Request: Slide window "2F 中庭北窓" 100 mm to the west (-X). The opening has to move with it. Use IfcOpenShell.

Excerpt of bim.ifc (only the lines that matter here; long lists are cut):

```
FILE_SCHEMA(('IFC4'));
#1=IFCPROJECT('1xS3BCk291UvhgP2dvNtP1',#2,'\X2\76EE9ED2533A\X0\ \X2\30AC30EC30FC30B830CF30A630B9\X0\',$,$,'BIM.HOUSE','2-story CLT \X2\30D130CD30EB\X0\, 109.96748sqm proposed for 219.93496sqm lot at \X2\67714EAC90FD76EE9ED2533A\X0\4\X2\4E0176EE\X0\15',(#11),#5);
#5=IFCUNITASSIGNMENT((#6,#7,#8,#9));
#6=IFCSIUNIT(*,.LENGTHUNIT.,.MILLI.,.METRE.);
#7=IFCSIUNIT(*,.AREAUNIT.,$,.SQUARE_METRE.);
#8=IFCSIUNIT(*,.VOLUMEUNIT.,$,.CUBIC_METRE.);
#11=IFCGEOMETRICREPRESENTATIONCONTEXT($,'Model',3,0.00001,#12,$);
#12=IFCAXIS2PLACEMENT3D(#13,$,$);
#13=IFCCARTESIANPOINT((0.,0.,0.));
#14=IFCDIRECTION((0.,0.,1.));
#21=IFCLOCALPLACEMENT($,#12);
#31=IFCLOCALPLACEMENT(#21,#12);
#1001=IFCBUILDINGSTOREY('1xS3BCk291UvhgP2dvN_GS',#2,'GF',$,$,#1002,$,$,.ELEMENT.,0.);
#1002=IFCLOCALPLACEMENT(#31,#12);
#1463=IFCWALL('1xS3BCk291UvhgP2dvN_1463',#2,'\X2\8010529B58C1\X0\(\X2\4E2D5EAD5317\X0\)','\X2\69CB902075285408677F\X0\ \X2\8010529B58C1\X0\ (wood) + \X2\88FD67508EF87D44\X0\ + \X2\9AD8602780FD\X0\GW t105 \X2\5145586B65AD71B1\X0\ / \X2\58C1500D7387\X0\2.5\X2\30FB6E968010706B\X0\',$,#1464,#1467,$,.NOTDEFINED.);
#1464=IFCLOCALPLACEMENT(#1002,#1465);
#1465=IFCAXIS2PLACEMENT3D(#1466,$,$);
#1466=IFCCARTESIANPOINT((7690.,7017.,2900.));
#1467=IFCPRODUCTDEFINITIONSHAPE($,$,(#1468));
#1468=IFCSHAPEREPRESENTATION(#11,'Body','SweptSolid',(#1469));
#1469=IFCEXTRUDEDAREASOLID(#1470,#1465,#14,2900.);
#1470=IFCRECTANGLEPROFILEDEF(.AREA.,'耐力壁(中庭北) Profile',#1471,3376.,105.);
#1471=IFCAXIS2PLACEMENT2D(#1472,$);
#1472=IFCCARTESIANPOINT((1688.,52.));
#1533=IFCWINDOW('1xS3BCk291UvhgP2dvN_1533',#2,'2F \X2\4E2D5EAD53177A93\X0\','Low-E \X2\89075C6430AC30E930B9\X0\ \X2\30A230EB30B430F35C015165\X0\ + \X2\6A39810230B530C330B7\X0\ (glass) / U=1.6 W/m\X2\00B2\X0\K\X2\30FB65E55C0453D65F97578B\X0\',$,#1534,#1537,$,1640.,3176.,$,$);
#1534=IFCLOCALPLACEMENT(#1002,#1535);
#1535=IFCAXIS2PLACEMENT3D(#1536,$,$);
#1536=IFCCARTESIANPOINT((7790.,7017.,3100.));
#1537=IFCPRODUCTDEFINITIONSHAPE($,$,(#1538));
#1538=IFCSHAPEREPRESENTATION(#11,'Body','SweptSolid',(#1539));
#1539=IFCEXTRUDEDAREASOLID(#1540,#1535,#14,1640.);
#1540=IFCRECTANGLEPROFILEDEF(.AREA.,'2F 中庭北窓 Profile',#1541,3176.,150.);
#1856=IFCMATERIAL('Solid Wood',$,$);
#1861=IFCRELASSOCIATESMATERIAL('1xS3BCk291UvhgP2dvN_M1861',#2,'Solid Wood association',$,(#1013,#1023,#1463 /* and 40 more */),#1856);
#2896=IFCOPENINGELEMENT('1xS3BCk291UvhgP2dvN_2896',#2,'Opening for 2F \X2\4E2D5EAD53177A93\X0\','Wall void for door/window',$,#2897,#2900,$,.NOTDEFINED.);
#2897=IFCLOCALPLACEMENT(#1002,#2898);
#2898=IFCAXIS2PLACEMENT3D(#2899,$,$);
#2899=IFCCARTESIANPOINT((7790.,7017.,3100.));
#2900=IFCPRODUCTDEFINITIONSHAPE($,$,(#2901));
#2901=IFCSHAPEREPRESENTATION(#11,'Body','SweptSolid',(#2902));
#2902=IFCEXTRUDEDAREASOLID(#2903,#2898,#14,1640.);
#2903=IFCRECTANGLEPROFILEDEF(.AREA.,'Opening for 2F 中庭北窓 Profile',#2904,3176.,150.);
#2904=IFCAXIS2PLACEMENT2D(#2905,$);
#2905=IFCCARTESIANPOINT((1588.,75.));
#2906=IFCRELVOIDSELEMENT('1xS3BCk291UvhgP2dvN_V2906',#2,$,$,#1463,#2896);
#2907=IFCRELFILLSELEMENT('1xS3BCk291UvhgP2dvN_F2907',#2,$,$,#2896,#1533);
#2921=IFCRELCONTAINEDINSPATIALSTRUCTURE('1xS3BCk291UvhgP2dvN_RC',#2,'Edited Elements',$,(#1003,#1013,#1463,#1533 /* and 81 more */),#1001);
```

```python
import ifcopenshell
import ifcopenshell.api.geometry
import ifcopenshell.util.placement
import ifcopenshell.util.unit

model = ifcopenshell.open("bim.ifc")
unit_scale = ifcopenshell.util.unit.calculate_unit_scale(model)

window = model.by_id(1533)
opening = window.FillsVoids[0].RelatingOpeningElement
wall = opening.VoidsElements[0].RelatingBuildingElement

wall_matrix = ifcopenshell.util.placement.get_local_placement(wall.ObjectPlacement)
shift = wall_matrix[:3, 0] * -0.1 / unit_scale
before = ifcopenshell.util.placement.get_local_placement(window.ObjectPlacement)[:3, 3].copy()

# The window is not placed relative to its opening, so move both.
for product in (opening, window):
    matrix = ifcopenshell.util.placement.get_local_placement(product.ObjectPlacement)
    matrix[:3, 3] += shift
    ifcopenshell.api.geometry.edit_object_placement(model, product=product, matrix=matrix, is_si=False)

after = ifcopenshell.util.placement.get_local_placement(window.ObjectPlacement)[:3, 3]
print("window moved by", (after - before).round(3) + 0.0)

model.write("bim_edited.ifc")
```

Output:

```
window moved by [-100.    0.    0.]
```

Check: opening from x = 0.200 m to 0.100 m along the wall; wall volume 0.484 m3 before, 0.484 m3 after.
